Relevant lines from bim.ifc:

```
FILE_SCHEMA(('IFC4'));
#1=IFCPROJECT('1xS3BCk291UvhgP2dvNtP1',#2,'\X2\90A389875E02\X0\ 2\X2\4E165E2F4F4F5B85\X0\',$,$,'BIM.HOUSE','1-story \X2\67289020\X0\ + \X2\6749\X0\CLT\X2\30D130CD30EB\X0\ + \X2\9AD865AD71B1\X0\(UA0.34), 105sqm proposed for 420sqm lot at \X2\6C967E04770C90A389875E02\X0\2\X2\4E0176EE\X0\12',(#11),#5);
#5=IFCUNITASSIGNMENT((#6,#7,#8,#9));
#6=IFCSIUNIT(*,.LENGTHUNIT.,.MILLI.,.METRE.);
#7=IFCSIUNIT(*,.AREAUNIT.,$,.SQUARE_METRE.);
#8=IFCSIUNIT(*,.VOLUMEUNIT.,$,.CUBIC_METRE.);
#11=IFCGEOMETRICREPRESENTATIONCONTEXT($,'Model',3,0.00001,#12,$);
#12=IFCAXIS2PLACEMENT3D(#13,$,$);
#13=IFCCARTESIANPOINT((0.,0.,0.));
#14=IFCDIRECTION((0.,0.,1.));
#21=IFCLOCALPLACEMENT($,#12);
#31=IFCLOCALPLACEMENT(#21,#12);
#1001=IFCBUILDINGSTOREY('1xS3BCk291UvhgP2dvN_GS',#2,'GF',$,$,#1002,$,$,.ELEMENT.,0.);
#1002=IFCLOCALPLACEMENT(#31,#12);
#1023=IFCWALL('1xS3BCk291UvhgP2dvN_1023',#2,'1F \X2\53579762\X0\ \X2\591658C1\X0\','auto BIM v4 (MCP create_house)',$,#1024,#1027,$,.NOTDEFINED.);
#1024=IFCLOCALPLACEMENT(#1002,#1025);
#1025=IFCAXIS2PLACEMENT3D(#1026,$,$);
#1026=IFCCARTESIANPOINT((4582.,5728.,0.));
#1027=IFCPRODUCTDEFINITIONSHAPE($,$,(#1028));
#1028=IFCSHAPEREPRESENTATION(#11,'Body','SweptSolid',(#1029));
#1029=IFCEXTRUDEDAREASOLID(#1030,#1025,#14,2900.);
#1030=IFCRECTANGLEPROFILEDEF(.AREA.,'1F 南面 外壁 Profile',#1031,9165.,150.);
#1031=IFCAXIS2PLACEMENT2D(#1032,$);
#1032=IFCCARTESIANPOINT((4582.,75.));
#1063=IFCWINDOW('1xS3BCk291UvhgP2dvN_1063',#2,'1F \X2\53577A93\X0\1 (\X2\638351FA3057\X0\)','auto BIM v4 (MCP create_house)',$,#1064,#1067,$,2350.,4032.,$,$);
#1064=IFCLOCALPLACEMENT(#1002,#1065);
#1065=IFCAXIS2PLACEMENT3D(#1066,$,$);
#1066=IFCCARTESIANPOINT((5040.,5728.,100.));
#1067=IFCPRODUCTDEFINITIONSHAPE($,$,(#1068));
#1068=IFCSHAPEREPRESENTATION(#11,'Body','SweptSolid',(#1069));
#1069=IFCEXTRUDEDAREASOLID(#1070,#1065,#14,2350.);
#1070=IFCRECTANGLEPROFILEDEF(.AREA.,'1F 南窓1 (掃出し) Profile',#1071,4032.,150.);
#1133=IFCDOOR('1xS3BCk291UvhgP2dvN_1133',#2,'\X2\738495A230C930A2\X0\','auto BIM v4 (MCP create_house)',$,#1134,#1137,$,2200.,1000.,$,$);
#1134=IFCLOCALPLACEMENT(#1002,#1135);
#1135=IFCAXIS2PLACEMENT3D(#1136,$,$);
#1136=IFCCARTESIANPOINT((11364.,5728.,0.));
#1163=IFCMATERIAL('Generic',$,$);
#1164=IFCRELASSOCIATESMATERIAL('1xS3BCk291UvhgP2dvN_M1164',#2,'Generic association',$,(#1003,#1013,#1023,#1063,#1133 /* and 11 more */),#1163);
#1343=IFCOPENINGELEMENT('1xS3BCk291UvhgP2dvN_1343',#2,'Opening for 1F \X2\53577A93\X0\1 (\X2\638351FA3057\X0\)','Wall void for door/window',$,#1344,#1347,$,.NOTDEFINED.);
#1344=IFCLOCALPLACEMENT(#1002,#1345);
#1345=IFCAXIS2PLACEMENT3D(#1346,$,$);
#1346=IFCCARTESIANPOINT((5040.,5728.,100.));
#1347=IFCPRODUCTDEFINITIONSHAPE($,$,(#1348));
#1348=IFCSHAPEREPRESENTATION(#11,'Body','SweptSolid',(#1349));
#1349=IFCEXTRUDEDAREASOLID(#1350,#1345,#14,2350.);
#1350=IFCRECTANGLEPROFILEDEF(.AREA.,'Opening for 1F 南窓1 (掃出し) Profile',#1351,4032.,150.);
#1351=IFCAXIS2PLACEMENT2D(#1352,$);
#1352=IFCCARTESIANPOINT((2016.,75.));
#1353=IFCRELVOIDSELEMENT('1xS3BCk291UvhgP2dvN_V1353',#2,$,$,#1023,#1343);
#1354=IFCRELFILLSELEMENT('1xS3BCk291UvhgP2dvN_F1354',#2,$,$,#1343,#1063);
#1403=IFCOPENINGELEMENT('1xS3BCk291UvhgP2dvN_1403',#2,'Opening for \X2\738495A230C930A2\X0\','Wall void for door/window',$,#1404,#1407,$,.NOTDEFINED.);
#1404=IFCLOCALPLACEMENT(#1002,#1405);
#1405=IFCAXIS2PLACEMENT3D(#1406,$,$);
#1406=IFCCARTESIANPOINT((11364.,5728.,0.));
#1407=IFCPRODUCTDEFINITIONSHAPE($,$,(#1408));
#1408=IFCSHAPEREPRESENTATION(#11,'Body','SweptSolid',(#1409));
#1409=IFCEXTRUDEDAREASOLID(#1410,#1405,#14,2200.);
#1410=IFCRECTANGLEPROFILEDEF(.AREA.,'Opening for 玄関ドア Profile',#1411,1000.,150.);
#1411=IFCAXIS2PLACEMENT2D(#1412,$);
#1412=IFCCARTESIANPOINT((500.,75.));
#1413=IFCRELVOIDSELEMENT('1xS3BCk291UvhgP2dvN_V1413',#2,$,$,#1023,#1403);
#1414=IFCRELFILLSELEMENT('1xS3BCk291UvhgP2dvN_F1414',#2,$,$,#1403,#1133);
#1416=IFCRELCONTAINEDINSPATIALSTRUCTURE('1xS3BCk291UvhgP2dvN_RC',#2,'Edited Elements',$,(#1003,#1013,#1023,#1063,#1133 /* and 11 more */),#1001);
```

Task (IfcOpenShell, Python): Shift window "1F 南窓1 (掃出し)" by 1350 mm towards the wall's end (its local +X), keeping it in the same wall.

```python
import ifcopenshell
import ifcopenshell.api.geometry
import ifcopenshell.util.placement
import ifcopenshell.util.unit

model = ifcopenshell.open("bim.ifc")
unit_scale = ifcopenshell.util.unit.calculate_unit_scale(model)

window = model.by_guid("1xS3BCk291UvhgP2dvN_1063")
opening = window.FillsVoids[0].RelatingOpeningElement
wall = opening.VoidsElements[0].RelatingBuildingElement

wall_matrix = ifcopenshell.util.placement.get_local_placement(wall.ObjectPlacement)
shift = wall_matrix[:3, 0] * 1.35 / unit_scale
before = ifcopenshell.util.placement.get_local_placement(window.ObjectPlacement)[:3, 3].copy()

# The window is not placed relative to its opening, so move both.
for product in (opening, window):
    matrix = ifcopenshell.util.placement.get_local_placement(product.ObjectPlacement)
    matrix[:3, 3] += shift
    ifcopenshell.api.geometry.edit_object_placement(model, product=product, matrix=matrix, is_si=False)

after = ifcopenshell.util.placement.get_local_placement(window.ObjectPlacement)[:3, 3]
print("window moved by", (after - before).round(3) + 0.0)

model.write("bim_rev.ifc")
```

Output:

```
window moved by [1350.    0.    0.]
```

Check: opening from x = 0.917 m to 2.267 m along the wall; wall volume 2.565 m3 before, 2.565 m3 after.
